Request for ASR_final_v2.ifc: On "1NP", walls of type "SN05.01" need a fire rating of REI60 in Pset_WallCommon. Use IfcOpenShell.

First a look at what the model holds.

```python
import ifcopenshell
import ifcopenshell.util.element

model = ifcopenshell.open("ASR_final_v2.ifc")
print(model.schema)
storey = next(s for s in model.by_type("IfcBuildingStorey") if s.Name == "1NP")
walls = [e for e in ifcopenshell.util.element.get_decomposition(storey) if e.is_a("IfcWall")]
seen = {}
for e in walls:
    element_type = ifcopenshell.util.element.get_type(e)
    key = (element_type.Name if element_type != e and element_type else None, ifcopenshell.util.element.get_pset(e, "Pset_WallCommon", "FireRating"))
    seen[key] = seen.get(key, 0) + 1
for (name, value), count in sorted(seen.items(), key=str):
    print(count, "x", name, "|", value)
```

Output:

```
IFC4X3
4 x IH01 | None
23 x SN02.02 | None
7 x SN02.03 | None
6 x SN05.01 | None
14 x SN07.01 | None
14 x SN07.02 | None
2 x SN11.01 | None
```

```python
import ifcopenshell
import ifcopenshell.api.pset
import ifcopenshell.util.element

model = ifcopenshell.open("ASR_final_v2.ifc")

storey = next(s for s in model.by_type("IfcBuildingStorey") if s.Name == "1NP")
walls = [e for e in ifcopenshell.util.element.get_decomposition(storey) if e.is_a("IfcWall")]

count = 0
for e in walls:
    element_type = ifcopenshell.util.element.get_type(e)
    if element_type in (None, e) or element_type.Name != "SN05.01":
        continue
    # add_pset returns the element's existing set when there is one.
    pset = ifcopenshell.api.pset.add_pset(model, product=e, name="Pset_WallCommon")
    ifcopenshell.api.pset.edit_pset(model, pset=pset, properties={"FireRating": "REI60"})
    count += 1

print(count, "walls updated")

model.write("ASR_final_v2-out.ifc")
```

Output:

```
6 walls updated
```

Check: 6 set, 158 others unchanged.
